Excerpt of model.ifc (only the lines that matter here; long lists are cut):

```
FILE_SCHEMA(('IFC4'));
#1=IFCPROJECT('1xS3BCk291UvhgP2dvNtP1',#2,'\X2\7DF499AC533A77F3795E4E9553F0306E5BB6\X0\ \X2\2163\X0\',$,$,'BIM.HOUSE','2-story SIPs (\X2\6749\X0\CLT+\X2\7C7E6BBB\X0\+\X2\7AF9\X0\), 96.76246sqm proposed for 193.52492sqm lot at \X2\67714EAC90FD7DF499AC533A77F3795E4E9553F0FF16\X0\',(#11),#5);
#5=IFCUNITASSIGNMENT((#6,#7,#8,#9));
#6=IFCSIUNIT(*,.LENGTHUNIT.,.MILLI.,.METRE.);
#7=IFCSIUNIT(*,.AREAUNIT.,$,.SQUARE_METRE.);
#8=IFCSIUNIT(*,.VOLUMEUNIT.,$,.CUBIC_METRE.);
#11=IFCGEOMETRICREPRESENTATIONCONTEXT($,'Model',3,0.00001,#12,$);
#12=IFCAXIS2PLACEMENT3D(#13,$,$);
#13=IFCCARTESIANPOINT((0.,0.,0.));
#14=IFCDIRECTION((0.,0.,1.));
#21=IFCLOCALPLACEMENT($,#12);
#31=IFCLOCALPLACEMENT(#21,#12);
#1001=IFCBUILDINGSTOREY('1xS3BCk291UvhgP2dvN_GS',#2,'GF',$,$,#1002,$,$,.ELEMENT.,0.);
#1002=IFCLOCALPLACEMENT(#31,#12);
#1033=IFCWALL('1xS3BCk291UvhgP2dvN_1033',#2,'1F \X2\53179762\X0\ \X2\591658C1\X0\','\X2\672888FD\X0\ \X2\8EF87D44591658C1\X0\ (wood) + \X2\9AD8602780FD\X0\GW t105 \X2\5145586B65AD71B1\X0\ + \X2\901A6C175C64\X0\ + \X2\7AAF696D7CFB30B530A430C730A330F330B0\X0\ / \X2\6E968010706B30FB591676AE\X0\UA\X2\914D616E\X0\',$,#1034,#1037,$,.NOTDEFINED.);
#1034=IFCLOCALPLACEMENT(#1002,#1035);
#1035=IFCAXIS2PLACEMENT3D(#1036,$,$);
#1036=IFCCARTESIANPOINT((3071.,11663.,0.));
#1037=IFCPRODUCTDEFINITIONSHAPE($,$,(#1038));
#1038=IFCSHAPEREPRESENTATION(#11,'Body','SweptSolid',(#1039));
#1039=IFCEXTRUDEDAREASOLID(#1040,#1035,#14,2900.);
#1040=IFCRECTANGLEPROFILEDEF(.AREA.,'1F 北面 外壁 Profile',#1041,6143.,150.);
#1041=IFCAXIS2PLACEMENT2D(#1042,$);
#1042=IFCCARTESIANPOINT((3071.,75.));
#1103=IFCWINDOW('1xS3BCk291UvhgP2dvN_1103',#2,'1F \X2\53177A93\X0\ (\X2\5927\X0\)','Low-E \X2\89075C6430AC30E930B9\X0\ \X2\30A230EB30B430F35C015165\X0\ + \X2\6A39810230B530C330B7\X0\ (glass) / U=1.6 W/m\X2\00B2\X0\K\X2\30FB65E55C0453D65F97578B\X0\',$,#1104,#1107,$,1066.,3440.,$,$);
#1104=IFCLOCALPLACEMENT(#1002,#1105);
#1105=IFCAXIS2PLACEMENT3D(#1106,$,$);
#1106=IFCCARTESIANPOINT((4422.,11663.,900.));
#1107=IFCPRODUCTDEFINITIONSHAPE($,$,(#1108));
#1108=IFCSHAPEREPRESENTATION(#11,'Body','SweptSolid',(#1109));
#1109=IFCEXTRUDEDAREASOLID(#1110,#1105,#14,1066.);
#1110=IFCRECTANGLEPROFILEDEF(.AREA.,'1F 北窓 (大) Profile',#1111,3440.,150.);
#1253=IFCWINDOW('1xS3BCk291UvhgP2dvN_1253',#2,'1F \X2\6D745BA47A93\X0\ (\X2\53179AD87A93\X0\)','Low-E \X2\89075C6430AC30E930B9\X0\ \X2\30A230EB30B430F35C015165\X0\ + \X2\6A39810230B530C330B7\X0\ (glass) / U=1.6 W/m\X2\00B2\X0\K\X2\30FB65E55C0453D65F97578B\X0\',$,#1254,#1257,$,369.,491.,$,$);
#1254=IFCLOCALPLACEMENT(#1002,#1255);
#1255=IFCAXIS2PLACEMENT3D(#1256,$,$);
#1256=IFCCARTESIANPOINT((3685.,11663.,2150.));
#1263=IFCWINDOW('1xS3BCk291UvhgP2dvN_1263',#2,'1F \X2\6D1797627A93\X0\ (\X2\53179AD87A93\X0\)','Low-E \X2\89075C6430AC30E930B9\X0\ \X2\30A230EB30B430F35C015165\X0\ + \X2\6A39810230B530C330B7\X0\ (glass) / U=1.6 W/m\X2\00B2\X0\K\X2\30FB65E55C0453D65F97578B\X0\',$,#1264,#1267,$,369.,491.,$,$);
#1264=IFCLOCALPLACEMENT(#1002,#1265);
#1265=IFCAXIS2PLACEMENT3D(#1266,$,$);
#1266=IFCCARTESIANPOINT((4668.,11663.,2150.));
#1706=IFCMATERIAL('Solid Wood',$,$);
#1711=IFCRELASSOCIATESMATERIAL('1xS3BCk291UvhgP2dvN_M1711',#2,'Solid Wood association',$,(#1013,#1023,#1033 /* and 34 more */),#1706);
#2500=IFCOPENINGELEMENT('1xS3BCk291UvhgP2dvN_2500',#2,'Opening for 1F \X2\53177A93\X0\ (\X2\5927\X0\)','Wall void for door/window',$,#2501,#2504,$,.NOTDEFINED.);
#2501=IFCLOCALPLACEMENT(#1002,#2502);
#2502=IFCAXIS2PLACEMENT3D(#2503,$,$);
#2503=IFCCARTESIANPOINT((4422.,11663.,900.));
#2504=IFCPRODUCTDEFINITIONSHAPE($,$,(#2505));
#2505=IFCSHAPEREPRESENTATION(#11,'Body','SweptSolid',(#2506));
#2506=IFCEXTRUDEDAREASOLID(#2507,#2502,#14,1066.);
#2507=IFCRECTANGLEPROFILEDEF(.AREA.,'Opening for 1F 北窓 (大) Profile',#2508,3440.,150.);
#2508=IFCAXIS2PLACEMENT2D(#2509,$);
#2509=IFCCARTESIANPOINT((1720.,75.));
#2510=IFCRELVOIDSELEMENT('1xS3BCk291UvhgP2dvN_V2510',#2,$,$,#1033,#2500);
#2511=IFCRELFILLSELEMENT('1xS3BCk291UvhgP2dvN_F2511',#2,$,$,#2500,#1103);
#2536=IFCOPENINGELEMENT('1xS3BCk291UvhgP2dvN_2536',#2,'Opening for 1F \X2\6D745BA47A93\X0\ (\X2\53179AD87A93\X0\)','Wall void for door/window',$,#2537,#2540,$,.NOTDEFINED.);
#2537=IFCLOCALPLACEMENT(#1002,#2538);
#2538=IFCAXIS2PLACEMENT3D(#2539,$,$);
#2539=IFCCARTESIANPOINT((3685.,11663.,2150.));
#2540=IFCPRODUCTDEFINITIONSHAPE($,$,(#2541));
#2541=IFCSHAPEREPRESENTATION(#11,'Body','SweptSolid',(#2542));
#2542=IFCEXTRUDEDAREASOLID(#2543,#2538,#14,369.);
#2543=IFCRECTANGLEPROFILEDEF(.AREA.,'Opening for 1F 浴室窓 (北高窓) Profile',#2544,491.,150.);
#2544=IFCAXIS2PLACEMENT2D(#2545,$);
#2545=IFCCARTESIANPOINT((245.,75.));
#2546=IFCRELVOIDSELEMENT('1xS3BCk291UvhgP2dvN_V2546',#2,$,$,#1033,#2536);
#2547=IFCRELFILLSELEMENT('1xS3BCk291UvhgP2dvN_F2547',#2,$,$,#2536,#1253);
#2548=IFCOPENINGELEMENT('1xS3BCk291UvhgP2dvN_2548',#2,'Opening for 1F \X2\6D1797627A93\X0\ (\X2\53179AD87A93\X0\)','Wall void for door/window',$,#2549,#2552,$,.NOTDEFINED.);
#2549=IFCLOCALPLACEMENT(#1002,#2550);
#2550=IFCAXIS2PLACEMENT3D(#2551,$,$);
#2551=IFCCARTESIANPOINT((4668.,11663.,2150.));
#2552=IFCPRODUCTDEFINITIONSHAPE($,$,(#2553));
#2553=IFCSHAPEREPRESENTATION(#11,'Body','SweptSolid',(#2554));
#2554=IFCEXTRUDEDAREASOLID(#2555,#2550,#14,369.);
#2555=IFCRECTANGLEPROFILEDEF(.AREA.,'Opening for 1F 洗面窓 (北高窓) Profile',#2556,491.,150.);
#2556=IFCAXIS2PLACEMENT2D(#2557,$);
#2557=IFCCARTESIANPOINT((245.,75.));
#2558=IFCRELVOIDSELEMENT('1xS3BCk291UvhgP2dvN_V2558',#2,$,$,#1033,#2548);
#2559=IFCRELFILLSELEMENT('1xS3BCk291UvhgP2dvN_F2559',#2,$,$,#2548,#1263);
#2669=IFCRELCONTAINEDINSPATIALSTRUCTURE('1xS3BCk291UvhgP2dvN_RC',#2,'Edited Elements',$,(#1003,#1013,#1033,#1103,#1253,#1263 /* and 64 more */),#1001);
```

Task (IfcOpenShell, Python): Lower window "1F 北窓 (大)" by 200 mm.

```python
import numpy as np
import ifcopenshell
import ifcopenshell.api.geometry
import ifcopenshell.util.placement
import ifcopenshell.util.unit

model = ifcopenshell.open("model.ifc")
unit_scale = ifcopenshell.util.unit.calculate_unit_scale(model)

window = model.by_guid("1xS3BCk291UvhgP2dvN_1103")
opening = window.FillsVoids[0].RelatingOpeningElement
dz = -0.2 / unit_scale

shift = np.array([0.0, 0.0, dz])
# The window is not placed relative to its opening, so move both.
for product in (opening, window):
    matrix = ifcopenshell.util.placement.get_local_placement(product.ObjectPlacement)
    matrix[:3, 3] += shift
    ifcopenshell.api.geometry.edit_object_placement(model, product=product, matrix=matrix, is_si=False)

print(f"moved by {dz * unit_scale:+.3f} m")

model.write("model_rev.ifc")
```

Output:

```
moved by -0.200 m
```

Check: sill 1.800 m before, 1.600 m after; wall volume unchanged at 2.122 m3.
